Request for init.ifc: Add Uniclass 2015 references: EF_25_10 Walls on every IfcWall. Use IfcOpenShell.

First a look at what the model holds.

```python
import ifcopenshell

model = ifcopenshell.open("init.ifc")
print(model.schema)
print("classifications:", [c.Name for c in model.by_type("IfcClassification")])
for ifc_class in ("IfcDoor", "IfcRoof", "IfcStair", "IfcWall", "IfcWindow"):
    print(ifc_class, len(model.by_type(ifc_class)))
```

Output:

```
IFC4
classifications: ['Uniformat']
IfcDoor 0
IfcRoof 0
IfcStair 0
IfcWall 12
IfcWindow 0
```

```python
import ifcopenshell
import ifcopenshell.api.classification

model = ifcopenshell.open("init.ifc")

system = ifcopenshell.api.classification.add_classification(model, classification="Uniclass 2015")

codes = {
    "IfcWall": ("EF_25_10", "Walls"),
}
for ifc_class, (code, name) in codes.items():
    products = model.by_type(ifc_class)
    ifcopenshell.api.classification.add_reference(
        model, products=products, classification=system, identification=code, name=name
    )
    print(code, len(products))

model.write("init_updated.ifc")
```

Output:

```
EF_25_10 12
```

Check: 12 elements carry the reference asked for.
